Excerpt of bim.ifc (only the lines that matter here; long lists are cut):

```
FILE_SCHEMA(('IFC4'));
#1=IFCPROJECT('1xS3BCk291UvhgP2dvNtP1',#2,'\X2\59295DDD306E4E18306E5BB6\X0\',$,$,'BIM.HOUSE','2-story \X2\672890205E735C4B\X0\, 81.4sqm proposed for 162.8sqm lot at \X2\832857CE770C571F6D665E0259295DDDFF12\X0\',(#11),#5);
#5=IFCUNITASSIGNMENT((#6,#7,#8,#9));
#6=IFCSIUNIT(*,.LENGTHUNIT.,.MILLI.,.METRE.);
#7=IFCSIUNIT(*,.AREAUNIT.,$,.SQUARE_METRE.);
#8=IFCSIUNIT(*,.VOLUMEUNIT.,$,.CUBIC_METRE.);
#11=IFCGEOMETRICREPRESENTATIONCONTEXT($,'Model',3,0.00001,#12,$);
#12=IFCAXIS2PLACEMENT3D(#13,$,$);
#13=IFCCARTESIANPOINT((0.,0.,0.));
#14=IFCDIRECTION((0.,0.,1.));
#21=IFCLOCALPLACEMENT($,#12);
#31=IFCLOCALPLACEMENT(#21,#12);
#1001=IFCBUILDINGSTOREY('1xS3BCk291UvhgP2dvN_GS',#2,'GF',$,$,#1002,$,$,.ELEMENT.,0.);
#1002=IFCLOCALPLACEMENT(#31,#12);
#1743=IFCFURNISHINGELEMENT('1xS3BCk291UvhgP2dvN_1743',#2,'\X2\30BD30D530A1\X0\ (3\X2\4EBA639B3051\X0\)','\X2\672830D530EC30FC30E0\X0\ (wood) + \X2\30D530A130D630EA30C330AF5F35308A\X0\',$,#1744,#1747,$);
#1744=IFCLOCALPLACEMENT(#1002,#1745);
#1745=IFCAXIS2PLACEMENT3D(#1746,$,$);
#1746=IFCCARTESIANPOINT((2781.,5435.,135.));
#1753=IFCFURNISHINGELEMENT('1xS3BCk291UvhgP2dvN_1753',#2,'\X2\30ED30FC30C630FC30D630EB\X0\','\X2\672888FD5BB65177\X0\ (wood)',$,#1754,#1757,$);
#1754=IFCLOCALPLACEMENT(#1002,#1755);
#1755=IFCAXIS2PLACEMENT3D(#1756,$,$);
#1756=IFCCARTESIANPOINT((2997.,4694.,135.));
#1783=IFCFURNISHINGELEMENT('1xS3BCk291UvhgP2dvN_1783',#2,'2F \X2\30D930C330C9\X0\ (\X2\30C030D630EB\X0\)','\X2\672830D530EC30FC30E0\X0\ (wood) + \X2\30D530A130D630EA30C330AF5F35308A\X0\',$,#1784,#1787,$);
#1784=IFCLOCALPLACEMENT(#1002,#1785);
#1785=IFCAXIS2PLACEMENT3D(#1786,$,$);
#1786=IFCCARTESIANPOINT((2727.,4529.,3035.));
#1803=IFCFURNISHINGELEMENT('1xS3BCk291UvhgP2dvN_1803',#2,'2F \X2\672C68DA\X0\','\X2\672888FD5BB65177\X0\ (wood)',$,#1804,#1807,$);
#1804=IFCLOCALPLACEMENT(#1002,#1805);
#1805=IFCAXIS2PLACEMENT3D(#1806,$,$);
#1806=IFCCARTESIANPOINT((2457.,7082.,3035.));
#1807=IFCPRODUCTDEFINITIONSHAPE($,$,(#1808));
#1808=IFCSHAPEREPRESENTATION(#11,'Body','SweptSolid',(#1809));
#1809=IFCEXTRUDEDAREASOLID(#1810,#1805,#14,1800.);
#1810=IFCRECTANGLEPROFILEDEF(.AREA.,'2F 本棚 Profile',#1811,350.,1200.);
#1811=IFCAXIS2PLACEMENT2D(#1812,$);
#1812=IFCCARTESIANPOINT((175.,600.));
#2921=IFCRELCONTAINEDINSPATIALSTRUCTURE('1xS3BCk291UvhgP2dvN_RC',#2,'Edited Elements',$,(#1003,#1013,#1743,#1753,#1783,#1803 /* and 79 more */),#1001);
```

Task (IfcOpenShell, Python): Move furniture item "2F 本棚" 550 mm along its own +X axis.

```python
import ifcopenshell
import ifcopenshell.api.geometry
import ifcopenshell.util.placement
import ifcopenshell.util.unit

model = ifcopenshell.open("bim.ifc")
unit_scale = ifcopenshell.util.unit.calculate_unit_scale(model)

item = model.by_id(1803)
matrix = ifcopenshell.util.placement.get_local_placement(item.ObjectPlacement)
matrix[:3, 3] += matrix[:3, 0] * 0.55 / unit_scale
ifcopenshell.api.geometry.edit_object_placement(model, product=item, matrix=matrix, is_si=False)

print(ifcopenshell.util.placement.get_local_placement(item.ObjectPlacement).round(3) + 0.0)

model.write("bim_updated.ifc")
```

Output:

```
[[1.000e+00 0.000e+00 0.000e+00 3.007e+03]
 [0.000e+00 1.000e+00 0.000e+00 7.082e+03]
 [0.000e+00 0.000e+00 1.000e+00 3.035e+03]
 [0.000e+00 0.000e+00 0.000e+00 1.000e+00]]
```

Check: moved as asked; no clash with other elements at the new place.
